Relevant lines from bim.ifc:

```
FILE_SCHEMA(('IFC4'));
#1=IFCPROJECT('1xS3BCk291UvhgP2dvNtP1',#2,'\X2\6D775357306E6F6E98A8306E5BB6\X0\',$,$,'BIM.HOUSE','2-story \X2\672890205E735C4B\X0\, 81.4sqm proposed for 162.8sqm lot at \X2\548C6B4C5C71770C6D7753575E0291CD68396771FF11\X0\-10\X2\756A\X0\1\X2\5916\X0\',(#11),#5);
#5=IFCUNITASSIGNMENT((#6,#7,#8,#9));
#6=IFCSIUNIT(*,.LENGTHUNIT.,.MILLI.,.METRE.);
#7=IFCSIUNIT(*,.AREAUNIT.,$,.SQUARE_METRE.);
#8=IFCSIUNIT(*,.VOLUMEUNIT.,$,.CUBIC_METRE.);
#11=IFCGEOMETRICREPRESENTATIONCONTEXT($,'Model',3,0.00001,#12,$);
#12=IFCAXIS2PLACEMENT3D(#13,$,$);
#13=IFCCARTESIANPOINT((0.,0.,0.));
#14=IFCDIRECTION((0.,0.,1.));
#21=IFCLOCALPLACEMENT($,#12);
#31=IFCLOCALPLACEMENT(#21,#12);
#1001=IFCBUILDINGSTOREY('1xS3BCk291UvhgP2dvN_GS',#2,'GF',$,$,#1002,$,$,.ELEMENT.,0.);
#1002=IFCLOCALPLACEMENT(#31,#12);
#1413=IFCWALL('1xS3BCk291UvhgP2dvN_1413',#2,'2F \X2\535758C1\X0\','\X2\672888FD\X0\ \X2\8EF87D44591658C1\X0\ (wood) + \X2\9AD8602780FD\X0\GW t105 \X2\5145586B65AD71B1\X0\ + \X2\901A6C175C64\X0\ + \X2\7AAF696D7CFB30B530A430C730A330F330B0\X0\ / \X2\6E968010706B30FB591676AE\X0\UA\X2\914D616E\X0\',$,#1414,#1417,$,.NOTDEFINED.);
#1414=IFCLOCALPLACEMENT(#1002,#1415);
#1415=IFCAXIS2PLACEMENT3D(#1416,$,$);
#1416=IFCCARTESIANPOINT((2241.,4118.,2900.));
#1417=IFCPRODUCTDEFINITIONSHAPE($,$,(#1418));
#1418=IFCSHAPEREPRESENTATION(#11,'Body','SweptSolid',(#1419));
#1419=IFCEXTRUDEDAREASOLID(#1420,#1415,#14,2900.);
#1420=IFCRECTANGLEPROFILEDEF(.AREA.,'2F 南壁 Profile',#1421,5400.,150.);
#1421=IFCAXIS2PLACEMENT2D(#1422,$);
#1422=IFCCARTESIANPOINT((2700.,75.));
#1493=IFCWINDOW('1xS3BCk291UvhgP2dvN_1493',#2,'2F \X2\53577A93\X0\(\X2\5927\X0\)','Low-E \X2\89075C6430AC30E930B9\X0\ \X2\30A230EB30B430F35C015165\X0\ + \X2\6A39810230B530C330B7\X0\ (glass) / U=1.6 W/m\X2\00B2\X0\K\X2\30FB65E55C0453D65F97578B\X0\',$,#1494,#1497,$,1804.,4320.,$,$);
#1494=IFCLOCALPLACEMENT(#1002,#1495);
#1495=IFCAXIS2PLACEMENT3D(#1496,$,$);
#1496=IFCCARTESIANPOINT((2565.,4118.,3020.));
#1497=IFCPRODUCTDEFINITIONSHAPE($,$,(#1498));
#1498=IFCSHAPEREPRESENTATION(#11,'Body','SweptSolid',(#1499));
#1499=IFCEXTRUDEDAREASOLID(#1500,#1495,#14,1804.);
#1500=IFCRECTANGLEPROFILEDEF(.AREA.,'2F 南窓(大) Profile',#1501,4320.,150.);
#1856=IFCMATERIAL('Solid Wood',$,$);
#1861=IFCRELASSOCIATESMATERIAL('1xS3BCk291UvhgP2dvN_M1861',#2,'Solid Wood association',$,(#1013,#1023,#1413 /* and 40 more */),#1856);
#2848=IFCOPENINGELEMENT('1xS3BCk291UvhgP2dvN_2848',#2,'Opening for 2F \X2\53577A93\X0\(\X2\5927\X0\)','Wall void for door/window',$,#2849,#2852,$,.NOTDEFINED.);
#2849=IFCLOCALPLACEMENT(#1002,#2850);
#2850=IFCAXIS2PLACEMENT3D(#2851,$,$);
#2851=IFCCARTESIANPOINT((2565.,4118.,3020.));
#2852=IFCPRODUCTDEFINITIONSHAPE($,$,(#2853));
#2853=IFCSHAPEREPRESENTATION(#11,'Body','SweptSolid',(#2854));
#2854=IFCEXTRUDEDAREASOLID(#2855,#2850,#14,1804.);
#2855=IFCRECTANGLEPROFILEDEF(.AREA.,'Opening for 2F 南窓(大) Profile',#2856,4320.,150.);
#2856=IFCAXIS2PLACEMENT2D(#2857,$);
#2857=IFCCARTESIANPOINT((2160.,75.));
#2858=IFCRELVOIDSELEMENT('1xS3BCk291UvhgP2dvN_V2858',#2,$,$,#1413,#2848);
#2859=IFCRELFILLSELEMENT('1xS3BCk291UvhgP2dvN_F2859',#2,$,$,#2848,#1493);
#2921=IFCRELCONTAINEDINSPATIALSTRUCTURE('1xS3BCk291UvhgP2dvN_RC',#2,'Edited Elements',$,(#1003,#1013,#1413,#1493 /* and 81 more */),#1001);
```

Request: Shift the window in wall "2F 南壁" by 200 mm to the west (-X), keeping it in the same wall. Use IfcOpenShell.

```python
import ifcopenshell
import ifcopenshell.api.geometry
import ifcopenshell.util.placement

model = ifcopenshell.open("bim.ifc")

window = model.by_guid("1xS3BCk291UvhgP2dvN_1493")
opening = window.FillsVoids[0].RelatingOpeningElement
wall = opening.VoidsElements[0].RelatingBuildingElement

wall_matrix = ifcopenshell.util.placement.get_local_placement(wall.ObjectPlacement)
shift = wall_matrix[:3, 0] * -200.0
before = ifcopenshell.util.placement.get_local_placement(window.ObjectPlacement)[:3, 3].copy()

# The window is not placed relative to its opening, so move both.
for product in (opening, window):
    matrix = ifcopenshell.util.placement.get_local_placement(product.ObjectPlacement)
    matrix[:3, 3] += shift
    ifcopenshell.api.geometry.edit_object_placement(model, product=product, matrix=matrix, is_si=False)

after = ifcopenshell.util.placement.get_local_placement(window.ObjectPlacement)[:3, 3]
print("window moved by", (after - before).round(3) + 0.0)

model.write("bim_rev.ifc")
```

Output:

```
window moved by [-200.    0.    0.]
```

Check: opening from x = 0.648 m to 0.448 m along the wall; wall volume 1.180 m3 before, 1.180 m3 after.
